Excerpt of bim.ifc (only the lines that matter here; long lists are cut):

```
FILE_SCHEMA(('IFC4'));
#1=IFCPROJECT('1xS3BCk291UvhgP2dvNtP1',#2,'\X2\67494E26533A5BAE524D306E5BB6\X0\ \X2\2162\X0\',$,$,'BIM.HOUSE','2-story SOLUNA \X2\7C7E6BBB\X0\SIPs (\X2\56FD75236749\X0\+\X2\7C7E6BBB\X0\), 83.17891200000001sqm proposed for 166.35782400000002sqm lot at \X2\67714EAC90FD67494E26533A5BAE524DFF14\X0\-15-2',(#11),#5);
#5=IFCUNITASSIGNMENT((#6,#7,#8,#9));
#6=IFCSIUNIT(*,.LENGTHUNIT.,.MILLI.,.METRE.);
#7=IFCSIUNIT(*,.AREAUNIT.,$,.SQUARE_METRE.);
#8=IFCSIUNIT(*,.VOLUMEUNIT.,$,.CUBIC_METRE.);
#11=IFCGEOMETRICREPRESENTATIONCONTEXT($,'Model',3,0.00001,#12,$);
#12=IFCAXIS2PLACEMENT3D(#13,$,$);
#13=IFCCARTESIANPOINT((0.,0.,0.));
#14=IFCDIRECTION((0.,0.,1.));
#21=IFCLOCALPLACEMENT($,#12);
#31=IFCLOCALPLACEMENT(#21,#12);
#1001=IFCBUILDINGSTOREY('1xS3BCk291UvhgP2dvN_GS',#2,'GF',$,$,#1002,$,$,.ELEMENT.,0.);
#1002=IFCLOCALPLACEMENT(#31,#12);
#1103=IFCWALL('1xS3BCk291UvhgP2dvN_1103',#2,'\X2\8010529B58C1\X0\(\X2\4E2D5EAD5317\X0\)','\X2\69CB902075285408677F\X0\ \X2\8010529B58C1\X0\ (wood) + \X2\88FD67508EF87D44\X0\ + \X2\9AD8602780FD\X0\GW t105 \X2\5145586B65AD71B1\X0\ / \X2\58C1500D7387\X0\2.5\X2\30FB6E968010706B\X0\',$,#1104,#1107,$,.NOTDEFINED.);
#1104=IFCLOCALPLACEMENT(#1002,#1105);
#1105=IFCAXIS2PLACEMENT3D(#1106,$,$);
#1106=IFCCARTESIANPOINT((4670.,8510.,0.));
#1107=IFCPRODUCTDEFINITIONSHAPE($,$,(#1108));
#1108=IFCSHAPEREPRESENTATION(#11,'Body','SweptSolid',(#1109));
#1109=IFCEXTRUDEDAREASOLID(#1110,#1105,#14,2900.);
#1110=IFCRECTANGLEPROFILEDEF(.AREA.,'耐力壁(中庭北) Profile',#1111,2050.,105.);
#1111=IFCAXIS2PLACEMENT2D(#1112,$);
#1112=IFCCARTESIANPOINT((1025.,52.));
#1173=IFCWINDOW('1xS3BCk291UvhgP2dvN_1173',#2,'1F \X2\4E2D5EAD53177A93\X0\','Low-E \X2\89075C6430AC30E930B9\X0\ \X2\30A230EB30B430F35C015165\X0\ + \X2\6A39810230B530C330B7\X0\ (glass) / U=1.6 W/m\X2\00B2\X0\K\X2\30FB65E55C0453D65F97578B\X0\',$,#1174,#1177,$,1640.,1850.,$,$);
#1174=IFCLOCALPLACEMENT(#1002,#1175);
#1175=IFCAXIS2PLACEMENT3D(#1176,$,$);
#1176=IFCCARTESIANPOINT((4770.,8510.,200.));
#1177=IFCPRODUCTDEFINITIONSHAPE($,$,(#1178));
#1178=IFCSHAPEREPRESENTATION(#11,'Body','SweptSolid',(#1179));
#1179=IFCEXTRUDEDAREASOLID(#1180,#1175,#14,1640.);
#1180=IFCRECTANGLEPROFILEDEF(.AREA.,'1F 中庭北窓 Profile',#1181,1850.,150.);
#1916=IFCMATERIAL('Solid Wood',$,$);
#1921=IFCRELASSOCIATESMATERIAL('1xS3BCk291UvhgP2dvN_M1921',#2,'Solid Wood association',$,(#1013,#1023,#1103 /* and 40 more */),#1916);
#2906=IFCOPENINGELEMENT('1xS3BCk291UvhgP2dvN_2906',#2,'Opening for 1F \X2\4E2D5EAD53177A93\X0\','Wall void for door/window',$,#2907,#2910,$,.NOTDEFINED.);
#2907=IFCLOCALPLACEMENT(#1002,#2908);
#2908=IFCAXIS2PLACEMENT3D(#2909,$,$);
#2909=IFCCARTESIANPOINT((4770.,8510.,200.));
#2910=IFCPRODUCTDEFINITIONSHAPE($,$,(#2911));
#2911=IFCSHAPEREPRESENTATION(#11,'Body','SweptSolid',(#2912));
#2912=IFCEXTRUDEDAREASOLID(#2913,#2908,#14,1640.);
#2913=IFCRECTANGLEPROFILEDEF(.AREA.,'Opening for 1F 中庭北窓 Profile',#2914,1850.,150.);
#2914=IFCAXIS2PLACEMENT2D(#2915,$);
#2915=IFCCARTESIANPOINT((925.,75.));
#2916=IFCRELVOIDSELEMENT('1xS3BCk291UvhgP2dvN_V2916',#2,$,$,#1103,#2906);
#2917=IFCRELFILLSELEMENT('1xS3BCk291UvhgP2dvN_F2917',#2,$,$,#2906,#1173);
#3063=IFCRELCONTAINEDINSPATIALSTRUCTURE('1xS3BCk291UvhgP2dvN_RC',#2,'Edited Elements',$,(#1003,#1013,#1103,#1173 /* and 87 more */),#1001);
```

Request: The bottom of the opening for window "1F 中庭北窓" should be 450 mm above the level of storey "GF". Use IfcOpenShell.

```python
import numpy as np
import ifcopenshell
import ifcopenshell.api.geometry
import ifcopenshell.geom
import ifcopenshell.util.element
import ifcopenshell.util.placement
import ifcopenshell.util.shape
import ifcopenshell.util.unit

model = ifcopenshell.open("bim.ifc")
unit_scale = ifcopenshell.util.unit.calculate_unit_scale(model)

window = model.by_guid("1xS3BCk291UvhgP2dvN_1173")
opening = window.FillsVoids[0].RelatingOpeningElement
storey = ifcopenshell.util.element.get_container(window, ifc_class="IfcBuildingStorey")
level = ifcopenshell.util.placement.get_local_placement(storey.ObjectPlacement)[2, 3]

# The opening's origin need not be at the sill, so measure its lowest point.
shape = ifcopenshell.geom.create_shape(ifcopenshell.geom.settings(), opening)
bottom = ifcopenshell.util.shape.get_shape_bottom_elevation(shape, shape.geometry) / unit_scale
dz = level + 0.45 / unit_scale - bottom

shift = np.array([0.0, 0.0, dz])
# The window is not placed relative to its opening, so move both.
for product in (opening, window):
    matrix = ifcopenshell.util.placement.get_local_placement(product.ObjectPlacement)
    matrix[:3, 3] += shift
    ifcopenshell.api.geometry.edit_object_placement(model, product=product, matrix=matrix, is_si=False)

print(f"moved by {dz * unit_scale:+.3f} m")

model.write("bim_edited.ifc")
```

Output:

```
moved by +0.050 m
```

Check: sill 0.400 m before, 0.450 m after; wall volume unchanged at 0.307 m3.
